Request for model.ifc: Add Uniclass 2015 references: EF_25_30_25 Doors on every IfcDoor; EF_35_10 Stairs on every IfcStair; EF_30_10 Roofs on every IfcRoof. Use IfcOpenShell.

First a look at what the model holds.

```python
import ifcopenshell

model = ifcopenshell.open("model.ifc")
print(model.schema)
print("classifications:", [c.Name for c in model.by_type("IfcClassification")])
for ifc_class in ("IfcDoor", "IfcRoof", "IfcStair", "IfcWall", "IfcWindow"):
    print(ifc_class, len(model.by_type(ifc_class)))
```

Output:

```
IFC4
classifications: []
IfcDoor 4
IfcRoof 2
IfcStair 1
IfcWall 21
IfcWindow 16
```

```python
import ifcopenshell
import ifcopenshell.api.classification

model = ifcopenshell.open("model.ifc")

system = ifcopenshell.api.classification.add_classification(model, classification="Uniclass 2015")

codes = {
    "IfcDoor": ("EF_25_30_25", "Doors"),
    "IfcStair": ("EF_35_10", "Stairs"),
    "IfcRoof": ("EF_30_10", "Roofs"),
}
for ifc_class, (code, name) in codes.items():
    products = model.by_type(ifc_class)
    ifcopenshell.api.classification.add_reference(
        model, products=products, classification=system, identification=code, name=name
    )
    print(code, len(products))

model.write("model_edited.ifc")
```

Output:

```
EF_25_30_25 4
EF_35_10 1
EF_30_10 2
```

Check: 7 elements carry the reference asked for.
